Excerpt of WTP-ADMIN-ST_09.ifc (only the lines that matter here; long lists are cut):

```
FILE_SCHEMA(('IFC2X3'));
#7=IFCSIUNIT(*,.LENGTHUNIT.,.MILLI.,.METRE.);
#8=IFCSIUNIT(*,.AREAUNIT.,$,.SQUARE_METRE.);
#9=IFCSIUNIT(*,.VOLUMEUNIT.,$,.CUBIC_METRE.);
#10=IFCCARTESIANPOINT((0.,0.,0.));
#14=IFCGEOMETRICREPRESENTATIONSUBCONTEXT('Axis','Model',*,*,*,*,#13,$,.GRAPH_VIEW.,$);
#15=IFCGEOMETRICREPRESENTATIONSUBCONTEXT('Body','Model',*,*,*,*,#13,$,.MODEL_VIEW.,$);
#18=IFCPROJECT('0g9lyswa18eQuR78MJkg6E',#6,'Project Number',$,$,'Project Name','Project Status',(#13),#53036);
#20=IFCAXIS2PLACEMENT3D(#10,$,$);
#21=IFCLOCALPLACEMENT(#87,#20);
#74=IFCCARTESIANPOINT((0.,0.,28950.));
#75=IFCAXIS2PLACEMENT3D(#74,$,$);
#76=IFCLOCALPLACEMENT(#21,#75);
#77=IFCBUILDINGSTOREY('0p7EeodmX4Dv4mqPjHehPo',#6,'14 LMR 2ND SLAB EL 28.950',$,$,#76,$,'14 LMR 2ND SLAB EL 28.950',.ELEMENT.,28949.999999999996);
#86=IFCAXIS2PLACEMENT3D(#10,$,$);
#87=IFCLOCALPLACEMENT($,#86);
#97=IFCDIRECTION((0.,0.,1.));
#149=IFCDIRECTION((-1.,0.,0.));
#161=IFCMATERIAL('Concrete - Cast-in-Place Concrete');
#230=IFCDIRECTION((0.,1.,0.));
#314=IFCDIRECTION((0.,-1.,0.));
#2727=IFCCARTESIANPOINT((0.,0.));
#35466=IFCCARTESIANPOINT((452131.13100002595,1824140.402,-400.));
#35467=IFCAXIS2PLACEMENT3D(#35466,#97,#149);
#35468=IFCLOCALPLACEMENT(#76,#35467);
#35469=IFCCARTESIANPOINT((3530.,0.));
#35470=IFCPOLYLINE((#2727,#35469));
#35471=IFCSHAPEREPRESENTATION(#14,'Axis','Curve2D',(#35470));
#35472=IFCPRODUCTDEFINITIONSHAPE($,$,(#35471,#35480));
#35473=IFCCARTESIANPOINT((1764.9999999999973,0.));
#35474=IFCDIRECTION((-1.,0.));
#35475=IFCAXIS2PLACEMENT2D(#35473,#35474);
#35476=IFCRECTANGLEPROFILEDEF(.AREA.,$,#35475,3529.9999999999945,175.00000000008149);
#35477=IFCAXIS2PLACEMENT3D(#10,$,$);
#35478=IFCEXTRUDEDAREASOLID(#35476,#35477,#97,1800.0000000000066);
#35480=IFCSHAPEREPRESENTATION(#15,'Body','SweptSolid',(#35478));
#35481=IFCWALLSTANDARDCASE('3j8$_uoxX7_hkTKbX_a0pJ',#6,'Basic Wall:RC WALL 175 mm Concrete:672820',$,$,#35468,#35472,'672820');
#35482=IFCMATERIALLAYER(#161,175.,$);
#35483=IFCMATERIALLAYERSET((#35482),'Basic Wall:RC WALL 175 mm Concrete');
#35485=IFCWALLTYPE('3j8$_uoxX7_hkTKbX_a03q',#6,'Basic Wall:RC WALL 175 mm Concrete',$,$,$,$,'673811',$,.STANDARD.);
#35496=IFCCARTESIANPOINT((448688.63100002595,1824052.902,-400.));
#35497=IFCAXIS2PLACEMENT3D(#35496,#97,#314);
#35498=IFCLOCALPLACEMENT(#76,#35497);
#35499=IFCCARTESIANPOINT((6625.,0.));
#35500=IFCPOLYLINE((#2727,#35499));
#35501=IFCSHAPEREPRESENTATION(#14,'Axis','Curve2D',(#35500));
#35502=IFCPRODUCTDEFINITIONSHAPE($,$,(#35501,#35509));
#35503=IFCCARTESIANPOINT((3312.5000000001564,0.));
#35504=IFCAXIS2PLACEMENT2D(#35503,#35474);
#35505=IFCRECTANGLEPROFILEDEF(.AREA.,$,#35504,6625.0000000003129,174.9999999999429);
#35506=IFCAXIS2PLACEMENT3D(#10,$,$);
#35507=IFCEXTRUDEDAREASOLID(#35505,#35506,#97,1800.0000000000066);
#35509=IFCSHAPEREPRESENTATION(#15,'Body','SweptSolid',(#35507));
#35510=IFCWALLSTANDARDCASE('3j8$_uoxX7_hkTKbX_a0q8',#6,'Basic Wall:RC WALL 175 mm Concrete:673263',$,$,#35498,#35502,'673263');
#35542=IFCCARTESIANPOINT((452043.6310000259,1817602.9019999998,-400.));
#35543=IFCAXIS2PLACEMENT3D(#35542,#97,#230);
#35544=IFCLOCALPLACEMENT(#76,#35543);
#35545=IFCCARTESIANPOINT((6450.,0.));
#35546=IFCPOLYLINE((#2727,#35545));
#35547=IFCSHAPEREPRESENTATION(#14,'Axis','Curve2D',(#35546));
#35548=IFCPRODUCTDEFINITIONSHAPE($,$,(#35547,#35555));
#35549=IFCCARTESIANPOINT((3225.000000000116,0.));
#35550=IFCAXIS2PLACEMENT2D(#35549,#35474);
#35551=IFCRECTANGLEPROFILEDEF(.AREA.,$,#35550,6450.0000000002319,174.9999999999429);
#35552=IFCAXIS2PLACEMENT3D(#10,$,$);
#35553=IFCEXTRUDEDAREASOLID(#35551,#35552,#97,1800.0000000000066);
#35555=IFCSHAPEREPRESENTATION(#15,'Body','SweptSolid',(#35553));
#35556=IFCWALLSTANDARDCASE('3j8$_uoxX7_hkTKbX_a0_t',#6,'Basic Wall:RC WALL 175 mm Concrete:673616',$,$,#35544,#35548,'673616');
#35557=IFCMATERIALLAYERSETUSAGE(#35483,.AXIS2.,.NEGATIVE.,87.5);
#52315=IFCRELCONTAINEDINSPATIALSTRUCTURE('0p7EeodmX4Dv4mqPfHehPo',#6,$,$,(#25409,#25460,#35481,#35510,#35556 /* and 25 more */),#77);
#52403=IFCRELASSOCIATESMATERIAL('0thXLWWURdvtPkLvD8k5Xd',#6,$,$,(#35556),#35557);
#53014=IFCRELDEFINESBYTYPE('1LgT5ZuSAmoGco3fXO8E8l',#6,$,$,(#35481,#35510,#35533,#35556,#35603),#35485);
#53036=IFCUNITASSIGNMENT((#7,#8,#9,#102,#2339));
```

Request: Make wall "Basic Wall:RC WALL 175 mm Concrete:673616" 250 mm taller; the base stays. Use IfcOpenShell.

```python
import ifcopenshell
import ifcopenshell.geom
import ifcopenshell.util.representation
import ifcopenshell.util.shape

model = ifcopenshell.open("WTP-ADMIN-ST_09.ifc")
settings = ifcopenshell.geom.settings()


def volume(element):
    """Net volume in cubic metres, openings subtracted."""
    shape = ifcopenshell.geom.create_shape(settings, element)
    return ifcopenshell.util.shape.get_volume(shape.geometry)


wall = model.by_guid("3j8$_uoxX7_hkTKbX_a0_t")
before = volume(wall)

body = ifcopenshell.util.representation.get_representation(wall, "Model", "Body")
solid = body.Items[0]
old_height = solid.Depth
solid.Depth += 250.0
after = volume(wall)

print(f"height {old_height:g} -> {solid.Depth:g}, volume {before:.3f} -> {after:.3f} m3")

model.write("WTP-ADMIN-ST_09_updated.ifc")
```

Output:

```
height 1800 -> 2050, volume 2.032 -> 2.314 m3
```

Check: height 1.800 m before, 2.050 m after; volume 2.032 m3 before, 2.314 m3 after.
